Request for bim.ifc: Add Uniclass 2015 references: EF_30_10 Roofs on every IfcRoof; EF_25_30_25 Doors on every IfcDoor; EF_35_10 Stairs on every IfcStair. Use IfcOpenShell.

First a look at what the model holds.

```python
import ifcopenshell

model = ifcopenshell.open("bim.ifc")
print(model.schema)
print("classifications:", [c.Name for c in model.by_type("IfcClassification")])
for ifc_class in ("IfcDoor", "IfcRoof", "IfcStair", "IfcWall", "IfcWindow"):
    print(ifc_class, len(model.by_type(ifc_class)))
```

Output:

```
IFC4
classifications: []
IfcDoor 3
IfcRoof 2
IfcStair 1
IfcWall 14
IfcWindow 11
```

```python
import ifcopenshell
import ifcopenshell.api.classification

model = ifcopenshell.open("bim.ifc")

system = ifcopenshell.api.classification.add_classification(model, classification="Uniclass 2015")

codes = {
    "IfcRoof": ("EF_30_10", "Roofs"),
    "IfcDoor": ("EF_25_30_25", "Doors"),
    "IfcStair": ("EF_35_10", "Stairs"),
}
for ifc_class, (code, name) in codes.items():
    products = model.by_type(ifc_class)
    ifcopenshell.api.classification.add_reference(
        model, products=products, classification=system, identification=code, name=name
    )
    print(code, len(products))

model.write("bim_edited.ifc")
```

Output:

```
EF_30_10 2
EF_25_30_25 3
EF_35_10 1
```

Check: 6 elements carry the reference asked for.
